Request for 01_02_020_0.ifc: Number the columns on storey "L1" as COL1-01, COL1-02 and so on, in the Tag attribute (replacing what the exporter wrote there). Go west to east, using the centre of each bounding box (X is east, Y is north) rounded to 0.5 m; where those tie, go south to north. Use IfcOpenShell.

First a look at what the model holds.

```python
import ifcopenshell
import ifcopenshell.util.element
import ifcopenshell.util.placement

model = ifcopenshell.open("01_02_020_0.ifc")
print(model.schema)
storey = next(s for s in model.by_type("IfcBuildingStorey") if s.Name == "L1")
columns = [e for e in ifcopenshell.util.element.get_decomposition(storey) if e.is_a("IfcColumn")]
for e in sorted(columns, key=lambda e: e.id()):
    origin = ifcopenshell.util.placement.get_local_placement(e.ObjectPlacement)[:3, 3]
    print(e.id(), e.Tag, e.Name, origin.round(2) + 0.0, sep=" | ")
```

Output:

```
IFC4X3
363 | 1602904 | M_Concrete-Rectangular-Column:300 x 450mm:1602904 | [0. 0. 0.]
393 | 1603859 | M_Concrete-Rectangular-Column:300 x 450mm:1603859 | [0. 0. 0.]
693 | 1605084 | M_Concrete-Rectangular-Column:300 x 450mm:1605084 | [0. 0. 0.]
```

```python
import ifcopenshell
import ifcopenshell.geom
import ifcopenshell.util.element
import ifcopenshell.util.shape

model = ifcopenshell.open("01_02_020_0.ifc")
settings = ifcopenshell.geom.settings()
settings.set("use-world-coords", True)


def centre(element):
    shape = ifcopenshell.geom.create_shape(settings, element)
    return ifcopenshell.util.shape.get_bbox_centroid(shape.geometry)


storey = next(s for s in model.by_type("IfcBuildingStorey") if s.Name == "L1")
columns = [e for e in ifcopenshell.util.element.get_decomposition(storey) if e.is_a("IfcColumn")]

# Insertion points can sit at a corner or the storey origin, so sort by the geometry (in metres).
centres = {e: centre(e) for e in columns}
columns.sort(key=lambda e: (round(centres[e][0] / 0.5), centres[e][1]))

for i, e in enumerate(columns, start=1):
    number = f"COL1-{i:02d}"
    e.Tag = number
    print(e.id(), number)

model.write("01_02_020_0-out.ifc")
```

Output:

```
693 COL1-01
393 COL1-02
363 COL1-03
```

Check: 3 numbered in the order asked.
